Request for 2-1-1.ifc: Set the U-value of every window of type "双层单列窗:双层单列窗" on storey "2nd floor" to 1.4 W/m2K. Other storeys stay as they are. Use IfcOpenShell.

First a look at what the model holds.

```python
import ifcopenshell
import ifcopenshell.util.element

model = ifcopenshell.open("2-1-1.ifc")
print(model.schema)
storey = next(s for s in model.by_type("IfcBuildingStorey") if s.Name == "2nd floor")
windows = [e for e in ifcopenshell.util.element.get_decomposition(storey) if e.is_a("IfcWindow")]
seen = {}
for e in windows:
    element_type = ifcopenshell.util.element.get_type(e)
    key = (element_type.Name if element_type != e and element_type else None, ifcopenshell.util.element.get_pset(e, "Pset_WindowCommon", "ThermalTransmittance"))
    seen[key] = seen.get(key, 0) + 1
for (name, value), count in sorted(seen.items(), key=str):
    print(count, "x", name, "|", value)
```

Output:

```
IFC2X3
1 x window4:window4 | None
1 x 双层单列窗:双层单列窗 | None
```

```python
import ifcopenshell
import ifcopenshell.api.pset
import ifcopenshell.util.element

model = ifcopenshell.open("2-1-1.ifc")

storey = next(s for s in model.by_type("IfcBuildingStorey") if s.Name == "2nd floor")
windows = [e for e in ifcopenshell.util.element.get_decomposition(storey) if e.is_a("IfcWindow")]

count = 0
for e in windows:
    element_type = ifcopenshell.util.element.get_type(e)
    if element_type in (None, e) or element_type.Name != "双层单列窗:双层单列窗":
        continue
    # add_pset returns the element's existing set when there is one.
    pset = ifcopenshell.api.pset.add_pset(model, product=e, name="Pset_WindowCommon")
    ifcopenshell.api.pset.edit_pset(model, pset=pset, properties={"ThermalTransmittance": 1.4})
    count += 1

print(count, "windows updated")

model.write("2-1-1_edited.ifc")
```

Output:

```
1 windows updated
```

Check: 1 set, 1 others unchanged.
